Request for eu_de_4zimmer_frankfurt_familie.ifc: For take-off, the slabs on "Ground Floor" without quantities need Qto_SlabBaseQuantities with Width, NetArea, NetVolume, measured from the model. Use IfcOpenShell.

First a look at what the model holds.

```python
import ifcopenshell
import ifcopenshell.util.element
import ifcopenshell.util.unit

model = ifcopenshell.open("eu_de_4zimmer_frankfurt_familie.ifc")
print(model.schema)
for unit_type in ("LENGTHUNIT", "AREAUNIT", "VOLUMEUNIT"):
    print(unit_type, ifcopenshell.util.unit.calculate_unit_scale(model, unit_type))
storey = next(s for s in model.by_type("IfcBuildingStorey") if s.Name == "Ground Floor")
slabs = [e for e in ifcopenshell.util.element.get_decomposition(storey) if e.is_a("IfcSlab")]
for e in sorted(slabs, key=lambda e: e.id()):
    print(e.id(), e.is_a(), e.Name, list(ifcopenshell.util.element.get_psets(e, qtos_only=True)), sep=" | ")
```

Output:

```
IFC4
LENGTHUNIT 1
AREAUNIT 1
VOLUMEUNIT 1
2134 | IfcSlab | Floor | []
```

```python
import ifcopenshell
import ifcopenshell.api.pset
import ifcopenshell.geom
import ifcopenshell.util.element
import ifcopenshell.util.shape
import ifcopenshell.util.unit

model = ifcopenshell.open("eu_de_4zimmer_frankfurt_familie.ifc")
unit_scale = ifcopenshell.util.unit.calculate_unit_scale(model)
area_scale = ifcopenshell.util.unit.calculate_unit_scale(model, "AREAUNIT")
volume_scale = ifcopenshell.util.unit.calculate_unit_scale(model, "VOLUMEUNIT")
settings = ifcopenshell.geom.settings()

storey = next(s for s in model.by_type("IfcBuildingStorey") if s.Name == "Ground Floor")
slabs = [e for e in ifcopenshell.util.element.get_decomposition(storey) if e.is_a("IfcSlab")]

for e in sorted(slabs, key=lambda e: e.id()):
    if ifcopenshell.util.element.get_psets(e, qtos_only=True, should_inherit=False):
        continue
    # Geometry comes back in metres, in the element's own axes.
    shape = ifcopenshell.geom.create_shape(settings, e)
    values = {
        "Width": ifcopenshell.util.shape.get_z(shape.geometry) / unit_scale,
        "NetArea": ifcopenshell.util.shape.get_footprint_area(shape.geometry) / area_scale,
        "NetVolume": ifcopenshell.util.shape.get_volume(shape.geometry) / volume_scale,
    }
    qto = ifcopenshell.api.pset.add_qto(model, product=e, name="Qto_SlabBaseQuantities")
    ifcopenshell.api.pset.edit_qto(model, qto=qto, properties=values)
    print(e.id(), {k: round(v, 3) for k, v in values.items()})

model.write("eu_de_4zimmer_frankfurt_familie_updated.ifc")
```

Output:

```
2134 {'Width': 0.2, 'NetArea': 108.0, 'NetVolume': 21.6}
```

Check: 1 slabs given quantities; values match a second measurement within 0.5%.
